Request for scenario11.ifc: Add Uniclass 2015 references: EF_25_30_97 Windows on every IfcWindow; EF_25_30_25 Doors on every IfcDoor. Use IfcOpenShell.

First a look at what the model holds.

```python
import ifcopenshell

model = ifcopenshell.open("scenario11.ifc")
print(model.schema)
print("classifications:", [c.Name for c in model.by_type("IfcClassification")])
for ifc_class in ("IfcDoor", "IfcRoof", "IfcStair", "IfcWall", "IfcWindow"):
    print(ifc_class, len(model.by_type(ifc_class)))
```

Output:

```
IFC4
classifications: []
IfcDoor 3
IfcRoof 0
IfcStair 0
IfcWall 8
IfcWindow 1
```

```python
import ifcopenshell
import ifcopenshell.api.classification

model = ifcopenshell.open("scenario11.ifc")

system = ifcopenshell.api.classification.add_classification(model, classification="Uniclass 2015")

codes = {
    "IfcWindow": ("EF_25_30_97", "Windows"),
    "IfcDoor": ("EF_25_30_25", "Doors"),
}
for ifc_class, (code, name) in codes.items():
    products = model.by_type(ifc_class)
    ifcopenshell.api.classification.add_reference(
        model, products=products, classification=system, identification=code, name=name
    )
    print(code, len(products))

model.write("scenario11_updated.ifc")
```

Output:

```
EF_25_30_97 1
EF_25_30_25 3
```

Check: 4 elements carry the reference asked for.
